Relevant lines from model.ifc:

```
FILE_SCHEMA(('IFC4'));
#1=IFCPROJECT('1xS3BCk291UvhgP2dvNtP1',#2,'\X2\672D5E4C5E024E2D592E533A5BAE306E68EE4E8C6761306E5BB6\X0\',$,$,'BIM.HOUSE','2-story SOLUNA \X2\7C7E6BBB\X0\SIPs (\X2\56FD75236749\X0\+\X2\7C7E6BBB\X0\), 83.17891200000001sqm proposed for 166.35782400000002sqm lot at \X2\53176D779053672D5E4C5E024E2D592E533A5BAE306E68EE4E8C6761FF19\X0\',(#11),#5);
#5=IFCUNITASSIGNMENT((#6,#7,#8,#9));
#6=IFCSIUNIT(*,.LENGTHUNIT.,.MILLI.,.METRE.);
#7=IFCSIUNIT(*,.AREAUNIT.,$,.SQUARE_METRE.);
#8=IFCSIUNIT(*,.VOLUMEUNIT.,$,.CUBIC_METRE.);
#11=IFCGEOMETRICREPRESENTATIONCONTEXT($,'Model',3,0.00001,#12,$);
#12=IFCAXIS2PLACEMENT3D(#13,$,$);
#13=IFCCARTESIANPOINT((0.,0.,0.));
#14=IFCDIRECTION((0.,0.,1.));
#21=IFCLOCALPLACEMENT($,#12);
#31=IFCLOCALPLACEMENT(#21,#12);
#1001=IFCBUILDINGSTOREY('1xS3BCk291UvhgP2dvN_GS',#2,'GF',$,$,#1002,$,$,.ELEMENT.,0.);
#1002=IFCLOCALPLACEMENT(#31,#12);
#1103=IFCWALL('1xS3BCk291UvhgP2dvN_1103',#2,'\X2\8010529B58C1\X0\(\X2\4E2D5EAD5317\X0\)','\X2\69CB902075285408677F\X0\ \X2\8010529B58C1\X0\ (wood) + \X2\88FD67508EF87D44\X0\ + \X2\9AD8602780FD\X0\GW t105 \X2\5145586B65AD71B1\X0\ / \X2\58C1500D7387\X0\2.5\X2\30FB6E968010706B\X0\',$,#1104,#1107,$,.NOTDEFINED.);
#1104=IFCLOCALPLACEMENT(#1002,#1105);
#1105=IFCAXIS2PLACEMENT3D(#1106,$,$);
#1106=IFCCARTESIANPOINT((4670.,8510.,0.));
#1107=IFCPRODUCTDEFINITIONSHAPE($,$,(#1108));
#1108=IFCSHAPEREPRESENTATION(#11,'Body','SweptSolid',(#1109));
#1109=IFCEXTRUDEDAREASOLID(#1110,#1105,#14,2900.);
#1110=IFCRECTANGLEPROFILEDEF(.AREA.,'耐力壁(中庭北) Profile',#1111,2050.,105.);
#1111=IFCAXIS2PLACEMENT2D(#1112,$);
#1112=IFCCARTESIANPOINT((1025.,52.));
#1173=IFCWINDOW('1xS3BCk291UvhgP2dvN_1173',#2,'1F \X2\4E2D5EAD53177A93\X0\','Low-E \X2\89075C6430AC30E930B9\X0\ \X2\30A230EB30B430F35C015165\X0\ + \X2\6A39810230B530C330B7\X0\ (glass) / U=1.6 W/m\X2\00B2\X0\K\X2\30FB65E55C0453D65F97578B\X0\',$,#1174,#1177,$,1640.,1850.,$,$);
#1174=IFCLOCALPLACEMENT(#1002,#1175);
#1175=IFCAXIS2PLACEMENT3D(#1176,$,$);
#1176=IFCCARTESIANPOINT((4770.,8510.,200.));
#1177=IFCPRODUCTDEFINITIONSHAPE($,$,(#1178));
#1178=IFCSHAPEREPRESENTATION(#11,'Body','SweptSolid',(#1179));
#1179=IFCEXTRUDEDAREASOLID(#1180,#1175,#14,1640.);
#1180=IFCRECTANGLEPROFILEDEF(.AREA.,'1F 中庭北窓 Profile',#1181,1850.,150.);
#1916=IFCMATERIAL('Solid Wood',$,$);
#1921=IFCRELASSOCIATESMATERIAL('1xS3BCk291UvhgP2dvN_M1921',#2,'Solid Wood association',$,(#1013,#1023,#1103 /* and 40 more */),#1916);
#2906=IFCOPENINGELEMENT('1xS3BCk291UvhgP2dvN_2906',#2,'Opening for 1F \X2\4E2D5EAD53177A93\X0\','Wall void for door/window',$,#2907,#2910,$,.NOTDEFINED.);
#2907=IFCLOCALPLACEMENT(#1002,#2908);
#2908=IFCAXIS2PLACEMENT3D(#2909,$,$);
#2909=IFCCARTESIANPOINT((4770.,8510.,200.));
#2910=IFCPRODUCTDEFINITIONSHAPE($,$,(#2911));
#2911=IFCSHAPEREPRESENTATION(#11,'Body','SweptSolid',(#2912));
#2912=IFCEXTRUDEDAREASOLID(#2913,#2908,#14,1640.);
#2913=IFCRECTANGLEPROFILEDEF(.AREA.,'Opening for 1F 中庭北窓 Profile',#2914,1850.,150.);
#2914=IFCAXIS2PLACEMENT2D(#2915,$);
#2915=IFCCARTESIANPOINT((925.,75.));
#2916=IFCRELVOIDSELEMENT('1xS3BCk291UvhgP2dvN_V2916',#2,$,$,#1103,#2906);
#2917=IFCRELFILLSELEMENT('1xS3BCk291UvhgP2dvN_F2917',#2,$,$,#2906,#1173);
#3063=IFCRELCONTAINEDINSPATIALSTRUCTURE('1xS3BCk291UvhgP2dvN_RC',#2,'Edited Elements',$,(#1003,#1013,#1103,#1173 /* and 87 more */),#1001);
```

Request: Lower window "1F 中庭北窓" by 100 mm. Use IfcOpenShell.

```python
import numpy as np
import ifcopenshell
import ifcopenshell.api.geometry
import ifcopenshell.util.placement
import ifcopenshell.util.unit

model = ifcopenshell.open("model.ifc")
unit_scale = ifcopenshell.util.unit.calculate_unit_scale(model)

window = model.by_guid("1xS3BCk291UvhgP2dvN_1173")
opening = window.FillsVoids[0].RelatingOpeningElement
dz = -100.0

shift = np.array([0.0, 0.0, dz])
# The window is not placed relative to its opening, so move both.
for product in (opening, window):
    matrix = ifcopenshell.util.placement.get_local_placement(product.ObjectPlacement)
    matrix[:3, 3] += shift
    ifcopenshell.api.geometry.edit_object_placement(model, product=product, matrix=matrix, is_si=False)

print(f"moved by {dz * unit_scale:+.3f} m")

model.write("model_v2.ifc")
```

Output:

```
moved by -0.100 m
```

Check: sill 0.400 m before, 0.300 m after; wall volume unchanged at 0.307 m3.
